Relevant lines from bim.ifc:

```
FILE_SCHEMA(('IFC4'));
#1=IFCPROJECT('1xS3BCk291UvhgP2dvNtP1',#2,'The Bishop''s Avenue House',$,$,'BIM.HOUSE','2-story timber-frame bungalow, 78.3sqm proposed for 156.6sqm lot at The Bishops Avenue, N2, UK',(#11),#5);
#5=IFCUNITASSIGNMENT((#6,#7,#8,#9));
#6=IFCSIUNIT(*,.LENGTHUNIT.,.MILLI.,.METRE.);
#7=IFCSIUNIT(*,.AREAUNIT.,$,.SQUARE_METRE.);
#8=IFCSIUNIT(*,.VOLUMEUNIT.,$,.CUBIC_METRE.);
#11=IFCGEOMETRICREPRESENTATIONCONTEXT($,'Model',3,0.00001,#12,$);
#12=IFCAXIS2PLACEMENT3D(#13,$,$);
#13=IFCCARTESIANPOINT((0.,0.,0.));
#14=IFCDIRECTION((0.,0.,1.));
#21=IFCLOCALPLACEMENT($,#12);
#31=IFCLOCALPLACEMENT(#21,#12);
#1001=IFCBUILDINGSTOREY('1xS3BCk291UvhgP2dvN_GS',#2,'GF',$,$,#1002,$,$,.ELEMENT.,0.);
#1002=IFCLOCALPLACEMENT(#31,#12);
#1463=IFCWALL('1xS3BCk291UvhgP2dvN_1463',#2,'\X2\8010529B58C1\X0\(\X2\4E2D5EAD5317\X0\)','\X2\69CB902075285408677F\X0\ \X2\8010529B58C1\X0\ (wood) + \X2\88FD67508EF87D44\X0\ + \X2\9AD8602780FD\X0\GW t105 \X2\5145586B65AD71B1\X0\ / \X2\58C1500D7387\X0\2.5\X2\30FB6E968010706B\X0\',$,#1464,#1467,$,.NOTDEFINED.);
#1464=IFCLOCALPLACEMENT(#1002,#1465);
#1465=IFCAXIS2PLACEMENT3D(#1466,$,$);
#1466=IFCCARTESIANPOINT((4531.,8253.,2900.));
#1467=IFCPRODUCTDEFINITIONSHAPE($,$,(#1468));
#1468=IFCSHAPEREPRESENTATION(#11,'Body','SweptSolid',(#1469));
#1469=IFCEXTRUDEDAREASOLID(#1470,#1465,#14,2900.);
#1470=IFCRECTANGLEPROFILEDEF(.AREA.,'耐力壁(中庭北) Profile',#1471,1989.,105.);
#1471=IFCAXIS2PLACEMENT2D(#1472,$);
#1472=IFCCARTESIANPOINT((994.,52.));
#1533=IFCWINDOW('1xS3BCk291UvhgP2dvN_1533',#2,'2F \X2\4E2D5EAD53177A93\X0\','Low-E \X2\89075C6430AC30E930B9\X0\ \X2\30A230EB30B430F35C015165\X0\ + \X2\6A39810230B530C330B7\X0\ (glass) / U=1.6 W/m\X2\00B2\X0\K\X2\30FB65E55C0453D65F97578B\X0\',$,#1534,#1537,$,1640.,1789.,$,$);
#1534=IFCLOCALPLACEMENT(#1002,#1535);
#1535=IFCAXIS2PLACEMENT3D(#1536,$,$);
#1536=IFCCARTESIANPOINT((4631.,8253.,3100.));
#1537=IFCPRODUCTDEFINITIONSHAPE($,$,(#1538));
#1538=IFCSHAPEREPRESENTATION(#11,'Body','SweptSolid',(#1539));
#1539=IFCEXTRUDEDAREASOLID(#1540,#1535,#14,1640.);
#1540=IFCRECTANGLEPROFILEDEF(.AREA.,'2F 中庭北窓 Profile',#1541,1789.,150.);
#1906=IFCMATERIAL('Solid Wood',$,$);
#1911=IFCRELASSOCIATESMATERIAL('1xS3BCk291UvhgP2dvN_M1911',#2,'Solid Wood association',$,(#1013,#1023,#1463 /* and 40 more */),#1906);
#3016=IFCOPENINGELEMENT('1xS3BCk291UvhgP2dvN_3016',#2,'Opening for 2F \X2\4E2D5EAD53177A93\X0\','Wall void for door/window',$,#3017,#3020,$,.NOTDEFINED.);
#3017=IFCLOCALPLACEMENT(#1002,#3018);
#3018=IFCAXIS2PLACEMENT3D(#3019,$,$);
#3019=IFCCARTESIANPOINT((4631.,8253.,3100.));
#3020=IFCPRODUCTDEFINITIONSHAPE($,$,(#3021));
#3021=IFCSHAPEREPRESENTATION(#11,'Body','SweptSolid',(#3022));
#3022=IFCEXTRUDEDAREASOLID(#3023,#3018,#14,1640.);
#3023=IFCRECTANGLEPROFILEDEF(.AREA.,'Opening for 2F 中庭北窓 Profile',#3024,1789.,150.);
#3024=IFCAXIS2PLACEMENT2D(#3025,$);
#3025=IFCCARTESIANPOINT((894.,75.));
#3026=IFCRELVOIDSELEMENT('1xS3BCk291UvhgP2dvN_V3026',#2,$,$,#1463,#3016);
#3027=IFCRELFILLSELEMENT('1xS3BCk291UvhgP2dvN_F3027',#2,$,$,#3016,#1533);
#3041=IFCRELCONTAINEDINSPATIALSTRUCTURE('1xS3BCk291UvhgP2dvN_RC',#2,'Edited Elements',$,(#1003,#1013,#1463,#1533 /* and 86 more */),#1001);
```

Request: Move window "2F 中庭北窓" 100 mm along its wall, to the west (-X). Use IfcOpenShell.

```python
import ifcopenshell
import ifcopenshell.api.geometry
import ifcopenshell.util.placement
import ifcopenshell.util.unit

model = ifcopenshell.open("bim.ifc")
unit_scale = ifcopenshell.util.unit.calculate_unit_scale(model)

window = model.by_guid("1xS3BCk291UvhgP2dvN_1533")
opening = window.FillsVoids[0].RelatingOpeningElement
wall = opening.VoidsElements[0].RelatingBuildingElement

wall_matrix = ifcopenshell.util.placement.get_local_placement(wall.ObjectPlacement)
shift = wall_matrix[:3, 0] * -0.1 / unit_scale
before = ifcopenshell.util.placement.get_local_placement(window.ObjectPlacement)[:3, 3].copy()

# The window is not placed relative to its opening, so move both.
for product in (opening, window):
    matrix = ifcopenshell.util.placement.get_local_placement(product.ObjectPlacement)
    matrix[:3, 3] += shift
    ifcopenshell.api.geometry.edit_object_placement(model, product=product, matrix=matrix, is_si=False)

after = ifcopenshell.util.placement.get_local_placement(window.ObjectPlacement)[:3, 3]
print("window moved by", (after - before).round(3) + 0.0)

model.write("bim-out.ifc")
```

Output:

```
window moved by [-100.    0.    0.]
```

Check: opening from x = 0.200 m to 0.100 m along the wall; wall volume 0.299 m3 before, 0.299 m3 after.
